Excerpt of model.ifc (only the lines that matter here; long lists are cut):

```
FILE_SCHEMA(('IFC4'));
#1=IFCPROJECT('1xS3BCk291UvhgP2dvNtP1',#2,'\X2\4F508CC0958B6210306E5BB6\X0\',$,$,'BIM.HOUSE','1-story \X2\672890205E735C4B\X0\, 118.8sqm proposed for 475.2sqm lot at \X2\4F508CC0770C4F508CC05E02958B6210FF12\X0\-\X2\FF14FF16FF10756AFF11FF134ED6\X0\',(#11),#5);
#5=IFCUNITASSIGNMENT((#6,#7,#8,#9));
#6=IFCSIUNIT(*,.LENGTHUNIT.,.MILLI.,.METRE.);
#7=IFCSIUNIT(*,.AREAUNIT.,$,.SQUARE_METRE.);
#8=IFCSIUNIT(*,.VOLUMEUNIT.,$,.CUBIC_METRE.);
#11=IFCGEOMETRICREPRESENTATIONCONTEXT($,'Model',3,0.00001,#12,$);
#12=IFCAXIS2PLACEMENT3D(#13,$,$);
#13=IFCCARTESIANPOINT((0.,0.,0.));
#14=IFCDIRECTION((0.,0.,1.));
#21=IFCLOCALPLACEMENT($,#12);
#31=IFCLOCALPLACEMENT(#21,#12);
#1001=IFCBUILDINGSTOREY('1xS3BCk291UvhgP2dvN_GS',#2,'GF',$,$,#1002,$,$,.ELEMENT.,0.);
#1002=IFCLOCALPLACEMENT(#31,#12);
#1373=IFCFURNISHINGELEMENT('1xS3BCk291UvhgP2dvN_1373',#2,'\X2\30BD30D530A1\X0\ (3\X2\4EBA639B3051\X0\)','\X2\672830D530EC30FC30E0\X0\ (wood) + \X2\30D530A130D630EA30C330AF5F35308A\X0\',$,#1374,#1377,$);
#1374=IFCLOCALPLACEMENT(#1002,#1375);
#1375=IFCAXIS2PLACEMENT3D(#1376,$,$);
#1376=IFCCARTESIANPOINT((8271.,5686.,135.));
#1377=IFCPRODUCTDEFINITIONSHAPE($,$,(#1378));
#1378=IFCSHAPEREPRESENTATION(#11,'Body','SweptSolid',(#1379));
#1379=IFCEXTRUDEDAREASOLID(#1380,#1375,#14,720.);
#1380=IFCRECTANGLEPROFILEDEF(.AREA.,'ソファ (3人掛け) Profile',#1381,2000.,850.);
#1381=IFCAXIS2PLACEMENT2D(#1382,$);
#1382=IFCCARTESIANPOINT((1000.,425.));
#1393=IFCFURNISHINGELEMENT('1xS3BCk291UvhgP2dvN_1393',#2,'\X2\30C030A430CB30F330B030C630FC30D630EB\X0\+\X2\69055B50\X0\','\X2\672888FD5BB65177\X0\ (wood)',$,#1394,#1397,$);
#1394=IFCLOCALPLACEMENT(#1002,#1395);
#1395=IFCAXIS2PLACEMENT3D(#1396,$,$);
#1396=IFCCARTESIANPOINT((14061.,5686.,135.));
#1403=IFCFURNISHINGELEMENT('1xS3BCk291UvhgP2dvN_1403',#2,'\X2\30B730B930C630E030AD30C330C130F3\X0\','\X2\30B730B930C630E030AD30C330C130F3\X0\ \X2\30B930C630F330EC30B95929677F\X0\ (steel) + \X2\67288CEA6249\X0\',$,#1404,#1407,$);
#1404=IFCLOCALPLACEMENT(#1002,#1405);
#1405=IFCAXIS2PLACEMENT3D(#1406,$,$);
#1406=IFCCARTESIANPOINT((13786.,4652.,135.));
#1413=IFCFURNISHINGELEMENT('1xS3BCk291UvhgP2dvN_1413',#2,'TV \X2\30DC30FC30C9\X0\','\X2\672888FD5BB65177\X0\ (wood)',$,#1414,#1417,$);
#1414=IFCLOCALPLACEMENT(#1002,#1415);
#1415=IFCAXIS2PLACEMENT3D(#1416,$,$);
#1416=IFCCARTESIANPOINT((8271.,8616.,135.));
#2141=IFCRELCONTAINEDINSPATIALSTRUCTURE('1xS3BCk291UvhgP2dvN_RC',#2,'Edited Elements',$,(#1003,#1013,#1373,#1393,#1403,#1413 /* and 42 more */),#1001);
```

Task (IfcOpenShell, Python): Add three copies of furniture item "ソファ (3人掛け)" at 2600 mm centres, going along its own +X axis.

```python
import ifcopenshell
import ifcopenshell.api.geometry
import ifcopenshell.api.root
import ifcopenshell.util.element
import ifcopenshell.util.placement
import ifcopenshell.util.unit

model = ifcopenshell.open("model.ifc")
unit_scale = ifcopenshell.util.unit.calculate_unit_scale(model)


def reuse_history(source, copy):
    """copy_class also copies each property set's owner history, people and application; keep the originals."""
    for rel in copy.IsDefinedBy:
        if rel.is_a("IfcRelDefinesByProperties") and (history := rel.RelatingPropertyDefinition.OwnerHistory):
            rel.RelatingPropertyDefinition.OwnerHistory = source.OwnerHistory
            ifcopenshell.util.element.remove_deep2(model, history)


source = model.by_guid("1xS3BCk291UvhgP2dvN_1373")
base = ifcopenshell.util.placement.get_local_placement(source.ObjectPlacement)
step = base[:3, 0] * 2.6 / unit_scale

for i in range(1, 4):
    copy = ifcopenshell.api.root.copy_class(model, product=source)
    copy.Representation = ifcopenshell.util.element.copy_deep(
        model, source.Representation, exclude=["IfcGeometricRepresentationContext", "IfcRepresentationMap"]
    )
    reuse_history(source, copy)
    matrix = base.copy()
    matrix[:3, 3] += i * step
    print("added at", matrix[:3, 3].round(3) + 0.0)
    ifcopenshell.api.geometry.edit_object_placement(model, product=copy, matrix=matrix, is_si=False)

model.write("model_rev.ifc")
```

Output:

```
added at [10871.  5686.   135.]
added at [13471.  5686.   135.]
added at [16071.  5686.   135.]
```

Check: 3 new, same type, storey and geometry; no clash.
